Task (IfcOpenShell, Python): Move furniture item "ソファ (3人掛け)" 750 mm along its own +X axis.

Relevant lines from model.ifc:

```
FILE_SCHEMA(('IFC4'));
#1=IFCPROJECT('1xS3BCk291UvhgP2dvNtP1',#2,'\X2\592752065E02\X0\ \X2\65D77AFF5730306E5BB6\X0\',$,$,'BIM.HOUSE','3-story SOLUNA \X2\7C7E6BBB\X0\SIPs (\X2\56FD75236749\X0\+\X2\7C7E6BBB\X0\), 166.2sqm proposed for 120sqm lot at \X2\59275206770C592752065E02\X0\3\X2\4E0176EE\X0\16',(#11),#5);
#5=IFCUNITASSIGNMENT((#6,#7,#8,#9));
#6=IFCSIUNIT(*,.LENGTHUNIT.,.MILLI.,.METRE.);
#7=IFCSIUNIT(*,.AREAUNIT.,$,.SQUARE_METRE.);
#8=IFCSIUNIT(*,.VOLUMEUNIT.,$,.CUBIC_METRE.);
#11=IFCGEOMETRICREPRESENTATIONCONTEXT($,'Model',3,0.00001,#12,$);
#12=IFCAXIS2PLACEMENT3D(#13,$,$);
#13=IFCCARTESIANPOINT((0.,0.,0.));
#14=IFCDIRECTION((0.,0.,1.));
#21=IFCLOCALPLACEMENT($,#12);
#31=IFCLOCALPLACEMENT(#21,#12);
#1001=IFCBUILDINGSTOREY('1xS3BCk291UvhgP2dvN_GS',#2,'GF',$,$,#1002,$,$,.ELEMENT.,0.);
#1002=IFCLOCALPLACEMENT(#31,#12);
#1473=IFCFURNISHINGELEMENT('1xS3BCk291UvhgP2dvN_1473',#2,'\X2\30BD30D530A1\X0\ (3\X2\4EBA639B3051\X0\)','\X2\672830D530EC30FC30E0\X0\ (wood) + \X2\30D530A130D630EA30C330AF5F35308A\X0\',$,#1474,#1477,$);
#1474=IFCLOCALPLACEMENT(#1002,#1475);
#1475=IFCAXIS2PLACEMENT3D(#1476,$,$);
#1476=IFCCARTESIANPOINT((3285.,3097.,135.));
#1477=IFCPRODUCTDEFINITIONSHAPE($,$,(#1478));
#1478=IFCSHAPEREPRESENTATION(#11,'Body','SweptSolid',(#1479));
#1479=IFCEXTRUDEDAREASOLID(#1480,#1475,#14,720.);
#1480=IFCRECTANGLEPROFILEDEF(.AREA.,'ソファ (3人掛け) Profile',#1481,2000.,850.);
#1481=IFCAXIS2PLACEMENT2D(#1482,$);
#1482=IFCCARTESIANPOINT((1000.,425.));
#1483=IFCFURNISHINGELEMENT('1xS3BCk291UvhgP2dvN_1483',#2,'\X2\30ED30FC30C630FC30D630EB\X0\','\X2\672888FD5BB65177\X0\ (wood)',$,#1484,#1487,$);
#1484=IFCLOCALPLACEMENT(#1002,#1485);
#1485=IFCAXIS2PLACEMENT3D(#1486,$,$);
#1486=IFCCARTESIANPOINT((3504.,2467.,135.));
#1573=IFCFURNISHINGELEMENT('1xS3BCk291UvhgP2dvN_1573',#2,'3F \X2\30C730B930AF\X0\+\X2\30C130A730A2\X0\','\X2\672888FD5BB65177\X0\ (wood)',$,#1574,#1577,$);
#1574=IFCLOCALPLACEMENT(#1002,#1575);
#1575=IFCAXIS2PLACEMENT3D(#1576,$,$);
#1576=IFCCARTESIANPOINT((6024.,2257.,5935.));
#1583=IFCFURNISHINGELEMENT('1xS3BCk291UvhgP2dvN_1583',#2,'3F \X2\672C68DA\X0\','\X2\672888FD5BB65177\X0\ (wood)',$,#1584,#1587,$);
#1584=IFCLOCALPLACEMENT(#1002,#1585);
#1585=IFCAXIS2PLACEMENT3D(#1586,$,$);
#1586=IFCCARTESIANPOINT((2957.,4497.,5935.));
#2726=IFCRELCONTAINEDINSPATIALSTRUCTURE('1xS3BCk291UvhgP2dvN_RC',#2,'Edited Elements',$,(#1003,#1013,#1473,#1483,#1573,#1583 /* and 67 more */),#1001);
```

```python
import ifcopenshell
import ifcopenshell.api.geometry
import ifcopenshell.util.placement
import ifcopenshell.util.unit

model = ifcopenshell.open("model.ifc")
unit_scale = ifcopenshell.util.unit.calculate_unit_scale(model)

item = model.by_guid("1xS3BCk291UvhgP2dvN_1473")
matrix = ifcopenshell.util.placement.get_local_placement(item.ObjectPlacement)
matrix[:3, 3] += matrix[:3, 0] * 0.75 / unit_scale
ifcopenshell.api.geometry.edit_object_placement(model, product=item, matrix=matrix, is_si=False)

print(ifcopenshell.util.placement.get_local_placement(item.ObjectPlacement).round(3) + 0.0)

model.write("model_v2.ifc")
```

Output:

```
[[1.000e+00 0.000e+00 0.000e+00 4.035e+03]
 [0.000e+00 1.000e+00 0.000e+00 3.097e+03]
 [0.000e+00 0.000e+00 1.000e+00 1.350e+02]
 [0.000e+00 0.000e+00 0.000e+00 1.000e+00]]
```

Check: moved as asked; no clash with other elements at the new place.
